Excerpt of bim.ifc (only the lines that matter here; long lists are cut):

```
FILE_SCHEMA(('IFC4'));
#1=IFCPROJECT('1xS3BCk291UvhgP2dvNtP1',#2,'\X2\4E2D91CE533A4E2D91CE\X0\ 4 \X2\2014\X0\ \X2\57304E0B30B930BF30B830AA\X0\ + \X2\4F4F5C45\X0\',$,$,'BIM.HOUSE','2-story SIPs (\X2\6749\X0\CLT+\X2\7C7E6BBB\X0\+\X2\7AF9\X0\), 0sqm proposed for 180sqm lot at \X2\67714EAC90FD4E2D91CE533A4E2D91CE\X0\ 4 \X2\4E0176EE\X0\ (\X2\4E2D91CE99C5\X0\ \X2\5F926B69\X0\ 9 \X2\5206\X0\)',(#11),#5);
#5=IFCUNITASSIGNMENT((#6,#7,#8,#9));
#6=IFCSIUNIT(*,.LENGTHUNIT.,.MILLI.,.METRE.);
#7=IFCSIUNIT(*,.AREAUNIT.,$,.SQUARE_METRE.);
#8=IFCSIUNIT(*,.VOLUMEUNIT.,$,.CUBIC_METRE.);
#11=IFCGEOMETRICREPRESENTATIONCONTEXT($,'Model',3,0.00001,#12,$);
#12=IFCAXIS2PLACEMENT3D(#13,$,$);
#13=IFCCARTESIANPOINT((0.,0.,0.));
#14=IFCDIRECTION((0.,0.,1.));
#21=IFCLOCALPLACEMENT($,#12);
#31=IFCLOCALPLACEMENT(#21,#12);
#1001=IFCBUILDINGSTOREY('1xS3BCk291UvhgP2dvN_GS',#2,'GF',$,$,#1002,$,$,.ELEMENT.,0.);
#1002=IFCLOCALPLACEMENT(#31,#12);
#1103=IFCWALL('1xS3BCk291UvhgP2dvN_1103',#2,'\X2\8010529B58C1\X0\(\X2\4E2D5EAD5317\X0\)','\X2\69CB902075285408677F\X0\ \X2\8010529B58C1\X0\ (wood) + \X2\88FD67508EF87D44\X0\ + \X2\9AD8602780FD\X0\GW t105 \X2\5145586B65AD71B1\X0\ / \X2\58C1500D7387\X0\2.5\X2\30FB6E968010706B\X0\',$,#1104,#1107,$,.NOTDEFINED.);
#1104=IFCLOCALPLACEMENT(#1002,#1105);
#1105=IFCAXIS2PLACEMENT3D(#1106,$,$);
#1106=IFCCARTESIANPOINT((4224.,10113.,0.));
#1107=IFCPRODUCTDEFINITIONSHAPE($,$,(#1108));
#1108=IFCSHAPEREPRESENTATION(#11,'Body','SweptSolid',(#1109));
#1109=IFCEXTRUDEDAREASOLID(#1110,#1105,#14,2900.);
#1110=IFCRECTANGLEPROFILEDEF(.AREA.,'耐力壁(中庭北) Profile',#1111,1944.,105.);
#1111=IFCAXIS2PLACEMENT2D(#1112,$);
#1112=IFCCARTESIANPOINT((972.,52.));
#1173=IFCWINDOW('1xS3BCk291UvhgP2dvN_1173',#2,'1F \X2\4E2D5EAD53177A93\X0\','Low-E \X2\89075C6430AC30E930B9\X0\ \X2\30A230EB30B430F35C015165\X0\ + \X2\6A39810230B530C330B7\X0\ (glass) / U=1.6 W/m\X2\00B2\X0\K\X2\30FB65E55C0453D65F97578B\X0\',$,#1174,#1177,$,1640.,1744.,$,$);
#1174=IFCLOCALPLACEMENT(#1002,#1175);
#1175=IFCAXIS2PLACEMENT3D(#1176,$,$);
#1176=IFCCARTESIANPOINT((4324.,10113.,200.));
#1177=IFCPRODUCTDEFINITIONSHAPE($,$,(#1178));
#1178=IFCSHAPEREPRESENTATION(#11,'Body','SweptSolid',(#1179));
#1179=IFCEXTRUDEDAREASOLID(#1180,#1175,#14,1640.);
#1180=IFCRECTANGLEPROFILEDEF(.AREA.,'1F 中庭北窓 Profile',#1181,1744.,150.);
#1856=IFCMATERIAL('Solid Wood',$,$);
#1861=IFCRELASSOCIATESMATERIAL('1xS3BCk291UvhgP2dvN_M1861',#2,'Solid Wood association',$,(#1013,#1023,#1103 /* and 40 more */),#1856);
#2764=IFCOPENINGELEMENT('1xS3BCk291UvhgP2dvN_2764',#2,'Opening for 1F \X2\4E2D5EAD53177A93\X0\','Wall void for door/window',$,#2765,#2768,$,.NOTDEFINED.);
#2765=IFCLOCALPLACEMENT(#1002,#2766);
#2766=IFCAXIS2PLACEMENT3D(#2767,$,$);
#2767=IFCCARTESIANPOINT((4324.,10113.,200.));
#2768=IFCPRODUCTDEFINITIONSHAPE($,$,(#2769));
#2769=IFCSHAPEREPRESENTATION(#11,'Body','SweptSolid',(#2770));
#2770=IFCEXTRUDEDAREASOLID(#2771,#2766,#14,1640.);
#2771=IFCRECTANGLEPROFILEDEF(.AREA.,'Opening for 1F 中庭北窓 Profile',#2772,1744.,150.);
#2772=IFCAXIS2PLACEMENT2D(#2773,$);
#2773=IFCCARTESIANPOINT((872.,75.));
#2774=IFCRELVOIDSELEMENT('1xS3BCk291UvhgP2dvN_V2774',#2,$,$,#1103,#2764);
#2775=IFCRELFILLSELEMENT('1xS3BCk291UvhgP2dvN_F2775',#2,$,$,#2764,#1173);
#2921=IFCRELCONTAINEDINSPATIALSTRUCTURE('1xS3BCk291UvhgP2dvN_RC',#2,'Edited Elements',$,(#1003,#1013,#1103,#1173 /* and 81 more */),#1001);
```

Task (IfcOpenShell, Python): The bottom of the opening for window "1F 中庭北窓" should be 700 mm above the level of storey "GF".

```python
import numpy as np
import ifcopenshell
import ifcopenshell.api.geometry
import ifcopenshell.geom
import ifcopenshell.util.element
import ifcopenshell.util.placement
import ifcopenshell.util.shape
import ifcopenshell.util.unit

model = ifcopenshell.open("bim.ifc")
unit_scale = ifcopenshell.util.unit.calculate_unit_scale(model)

window = model.by_guid("1xS3BCk291UvhgP2dvN_1173")
opening = window.FillsVoids[0].RelatingOpeningElement
storey = ifcopenshell.util.element.get_container(window, ifc_class="IfcBuildingStorey")
level = ifcopenshell.util.placement.get_local_placement(storey.ObjectPlacement)[2, 3]

# The opening's origin need not be at the sill, so measure its lowest point.
shape = ifcopenshell.geom.create_shape(ifcopenshell.geom.settings(), opening)
bottom = ifcopenshell.util.shape.get_shape_bottom_elevation(shape, shape.geometry) / unit_scale
dz = level + 0.7 / unit_scale - bottom

shift = np.array([0.0, 0.0, dz])
# The window is not placed relative to its opening, so move both.
for product in (opening, window):
    matrix = ifcopenshell.util.placement.get_local_placement(product.ObjectPlacement)
    matrix[:3, 3] += shift
    ifcopenshell.api.geometry.edit_object_placement(model, product=product, matrix=matrix, is_si=False)

print(f"moved by {dz * unit_scale:+.3f} m")

model.write("bim_v2.ifc")
```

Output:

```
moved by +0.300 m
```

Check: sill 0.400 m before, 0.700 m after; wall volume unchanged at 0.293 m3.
